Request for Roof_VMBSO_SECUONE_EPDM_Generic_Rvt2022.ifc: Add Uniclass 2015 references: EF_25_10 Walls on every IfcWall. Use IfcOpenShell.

First a look at what the model holds.

```python
import ifcopenshell

model = ifcopenshell.open("Roof_VMBSO_SECUONE_EPDM_Generic_Rvt2022.ifc")
print(model.schema)
print("classifications:", [c.Name for c in model.by_type("IfcClassification")])
for ifc_class in ("IfcDoor", "IfcRoof", "IfcStair", "IfcWall", "IfcWindow"):
    print(ifc_class, len(model.by_type(ifc_class)))
```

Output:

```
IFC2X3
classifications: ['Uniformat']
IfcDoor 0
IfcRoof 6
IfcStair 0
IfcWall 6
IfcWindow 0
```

```python
import ifcopenshell
import ifcopenshell.api.classification

model = ifcopenshell.open("Roof_VMBSO_SECUONE_EPDM_Generic_Rvt2022.ifc")

# IFC2X3 requires Source and Edition and has no link from the project to the system.
system = model.create_entity("IfcClassification", Source="NBS", Edition="2015", Name="Uniclass 2015")

codes = {
    "IfcWall": ("EF_25_10", "Walls"),
}
for ifc_class, (code, name) in codes.items():
    products = model.by_type(ifc_class)
    ifcopenshell.api.classification.add_reference(
        model, products=products, classification=system, identification=code, name=name
    )
    print(code, len(products))

model.write("Roof_VMBSO_SECUONE_EPDM_Generic_Rvt2022_updated.ifc")
```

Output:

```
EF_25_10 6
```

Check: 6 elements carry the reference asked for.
